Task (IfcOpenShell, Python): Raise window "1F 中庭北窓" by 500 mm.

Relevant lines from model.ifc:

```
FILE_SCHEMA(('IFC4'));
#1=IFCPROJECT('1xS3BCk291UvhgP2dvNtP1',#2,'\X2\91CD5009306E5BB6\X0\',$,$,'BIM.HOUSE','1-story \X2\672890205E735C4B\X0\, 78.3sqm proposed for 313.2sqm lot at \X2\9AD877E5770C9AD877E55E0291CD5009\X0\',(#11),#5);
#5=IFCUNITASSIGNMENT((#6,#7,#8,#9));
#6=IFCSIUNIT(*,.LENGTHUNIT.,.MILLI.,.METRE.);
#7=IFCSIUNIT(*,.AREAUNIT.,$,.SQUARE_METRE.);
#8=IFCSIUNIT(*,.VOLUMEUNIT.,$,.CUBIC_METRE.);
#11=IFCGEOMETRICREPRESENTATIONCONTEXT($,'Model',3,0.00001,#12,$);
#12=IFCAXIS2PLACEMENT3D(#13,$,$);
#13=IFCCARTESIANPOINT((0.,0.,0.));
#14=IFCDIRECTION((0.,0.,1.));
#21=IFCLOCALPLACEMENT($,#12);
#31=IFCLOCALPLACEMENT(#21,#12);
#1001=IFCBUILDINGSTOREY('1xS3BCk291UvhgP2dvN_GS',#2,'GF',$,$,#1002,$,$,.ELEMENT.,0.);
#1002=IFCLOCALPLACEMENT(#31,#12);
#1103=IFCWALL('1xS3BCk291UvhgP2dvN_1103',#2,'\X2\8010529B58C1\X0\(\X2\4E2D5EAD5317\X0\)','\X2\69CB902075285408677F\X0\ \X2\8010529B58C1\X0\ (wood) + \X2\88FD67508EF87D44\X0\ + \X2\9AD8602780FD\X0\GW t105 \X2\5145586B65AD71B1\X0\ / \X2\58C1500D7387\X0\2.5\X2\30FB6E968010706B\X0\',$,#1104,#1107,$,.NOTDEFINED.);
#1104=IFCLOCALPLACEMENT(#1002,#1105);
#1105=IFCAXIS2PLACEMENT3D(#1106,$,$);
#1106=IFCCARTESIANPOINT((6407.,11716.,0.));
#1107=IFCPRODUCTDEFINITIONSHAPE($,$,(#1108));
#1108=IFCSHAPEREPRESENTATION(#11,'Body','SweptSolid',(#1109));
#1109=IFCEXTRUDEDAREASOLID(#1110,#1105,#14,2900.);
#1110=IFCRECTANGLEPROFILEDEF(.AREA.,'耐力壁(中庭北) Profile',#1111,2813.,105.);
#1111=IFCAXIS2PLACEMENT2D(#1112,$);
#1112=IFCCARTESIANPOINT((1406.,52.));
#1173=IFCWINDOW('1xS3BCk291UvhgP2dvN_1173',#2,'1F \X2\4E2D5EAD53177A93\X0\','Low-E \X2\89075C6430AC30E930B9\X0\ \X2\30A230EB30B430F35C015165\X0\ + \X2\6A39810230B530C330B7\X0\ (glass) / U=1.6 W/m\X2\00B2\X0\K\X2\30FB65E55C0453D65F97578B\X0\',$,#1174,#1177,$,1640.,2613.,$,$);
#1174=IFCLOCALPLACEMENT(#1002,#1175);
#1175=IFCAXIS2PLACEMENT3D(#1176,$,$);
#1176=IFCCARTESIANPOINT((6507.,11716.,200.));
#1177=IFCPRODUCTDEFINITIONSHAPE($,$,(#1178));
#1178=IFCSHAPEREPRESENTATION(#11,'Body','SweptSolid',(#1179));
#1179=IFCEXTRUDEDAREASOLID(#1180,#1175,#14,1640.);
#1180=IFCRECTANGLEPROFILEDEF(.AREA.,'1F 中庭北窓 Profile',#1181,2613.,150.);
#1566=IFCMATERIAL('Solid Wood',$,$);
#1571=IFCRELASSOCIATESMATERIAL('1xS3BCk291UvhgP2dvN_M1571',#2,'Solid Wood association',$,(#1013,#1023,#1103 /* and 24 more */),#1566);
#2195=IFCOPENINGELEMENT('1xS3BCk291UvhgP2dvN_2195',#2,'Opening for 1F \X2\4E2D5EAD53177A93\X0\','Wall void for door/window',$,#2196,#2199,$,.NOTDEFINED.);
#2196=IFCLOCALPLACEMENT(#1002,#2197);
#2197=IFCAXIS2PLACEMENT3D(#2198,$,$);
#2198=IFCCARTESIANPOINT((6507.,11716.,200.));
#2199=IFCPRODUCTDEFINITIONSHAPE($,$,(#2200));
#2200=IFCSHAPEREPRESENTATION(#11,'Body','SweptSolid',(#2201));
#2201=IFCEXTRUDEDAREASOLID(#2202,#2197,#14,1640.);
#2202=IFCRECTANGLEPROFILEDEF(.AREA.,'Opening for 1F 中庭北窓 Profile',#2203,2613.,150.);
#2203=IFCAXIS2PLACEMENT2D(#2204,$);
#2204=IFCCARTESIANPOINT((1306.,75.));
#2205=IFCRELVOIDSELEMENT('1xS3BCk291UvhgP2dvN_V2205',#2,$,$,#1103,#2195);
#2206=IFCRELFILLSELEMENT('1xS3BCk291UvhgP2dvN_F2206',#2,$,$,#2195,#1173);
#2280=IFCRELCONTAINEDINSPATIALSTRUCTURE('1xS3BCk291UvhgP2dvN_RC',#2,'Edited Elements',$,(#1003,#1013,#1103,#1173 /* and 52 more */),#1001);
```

```python
import numpy as np
import ifcopenshell
import ifcopenshell.api.geometry
import ifcopenshell.util.placement
import ifcopenshell.util.unit

model = ifcopenshell.open("model.ifc")
unit_scale = ifcopenshell.util.unit.calculate_unit_scale(model)

window = model.by_guid("1xS3BCk291UvhgP2dvN_1173")
opening = window.FillsVoids[0].RelatingOpeningElement
dz = 500.0

shift = np.array([0.0, 0.0, dz])
# The window is not placed relative to its opening, so move both.
for product in (opening, window):
    matrix = ifcopenshell.util.placement.get_local_placement(product.ObjectPlacement)
    matrix[:3, 3] += shift
    ifcopenshell.api.geometry.edit_object_placement(model, product=product, matrix=matrix, is_si=False)

print(f"moved by {dz * unit_scale:+.3f} m")

model.write("model_rev.ifc")
```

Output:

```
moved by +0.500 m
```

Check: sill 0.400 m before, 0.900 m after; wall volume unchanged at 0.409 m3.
